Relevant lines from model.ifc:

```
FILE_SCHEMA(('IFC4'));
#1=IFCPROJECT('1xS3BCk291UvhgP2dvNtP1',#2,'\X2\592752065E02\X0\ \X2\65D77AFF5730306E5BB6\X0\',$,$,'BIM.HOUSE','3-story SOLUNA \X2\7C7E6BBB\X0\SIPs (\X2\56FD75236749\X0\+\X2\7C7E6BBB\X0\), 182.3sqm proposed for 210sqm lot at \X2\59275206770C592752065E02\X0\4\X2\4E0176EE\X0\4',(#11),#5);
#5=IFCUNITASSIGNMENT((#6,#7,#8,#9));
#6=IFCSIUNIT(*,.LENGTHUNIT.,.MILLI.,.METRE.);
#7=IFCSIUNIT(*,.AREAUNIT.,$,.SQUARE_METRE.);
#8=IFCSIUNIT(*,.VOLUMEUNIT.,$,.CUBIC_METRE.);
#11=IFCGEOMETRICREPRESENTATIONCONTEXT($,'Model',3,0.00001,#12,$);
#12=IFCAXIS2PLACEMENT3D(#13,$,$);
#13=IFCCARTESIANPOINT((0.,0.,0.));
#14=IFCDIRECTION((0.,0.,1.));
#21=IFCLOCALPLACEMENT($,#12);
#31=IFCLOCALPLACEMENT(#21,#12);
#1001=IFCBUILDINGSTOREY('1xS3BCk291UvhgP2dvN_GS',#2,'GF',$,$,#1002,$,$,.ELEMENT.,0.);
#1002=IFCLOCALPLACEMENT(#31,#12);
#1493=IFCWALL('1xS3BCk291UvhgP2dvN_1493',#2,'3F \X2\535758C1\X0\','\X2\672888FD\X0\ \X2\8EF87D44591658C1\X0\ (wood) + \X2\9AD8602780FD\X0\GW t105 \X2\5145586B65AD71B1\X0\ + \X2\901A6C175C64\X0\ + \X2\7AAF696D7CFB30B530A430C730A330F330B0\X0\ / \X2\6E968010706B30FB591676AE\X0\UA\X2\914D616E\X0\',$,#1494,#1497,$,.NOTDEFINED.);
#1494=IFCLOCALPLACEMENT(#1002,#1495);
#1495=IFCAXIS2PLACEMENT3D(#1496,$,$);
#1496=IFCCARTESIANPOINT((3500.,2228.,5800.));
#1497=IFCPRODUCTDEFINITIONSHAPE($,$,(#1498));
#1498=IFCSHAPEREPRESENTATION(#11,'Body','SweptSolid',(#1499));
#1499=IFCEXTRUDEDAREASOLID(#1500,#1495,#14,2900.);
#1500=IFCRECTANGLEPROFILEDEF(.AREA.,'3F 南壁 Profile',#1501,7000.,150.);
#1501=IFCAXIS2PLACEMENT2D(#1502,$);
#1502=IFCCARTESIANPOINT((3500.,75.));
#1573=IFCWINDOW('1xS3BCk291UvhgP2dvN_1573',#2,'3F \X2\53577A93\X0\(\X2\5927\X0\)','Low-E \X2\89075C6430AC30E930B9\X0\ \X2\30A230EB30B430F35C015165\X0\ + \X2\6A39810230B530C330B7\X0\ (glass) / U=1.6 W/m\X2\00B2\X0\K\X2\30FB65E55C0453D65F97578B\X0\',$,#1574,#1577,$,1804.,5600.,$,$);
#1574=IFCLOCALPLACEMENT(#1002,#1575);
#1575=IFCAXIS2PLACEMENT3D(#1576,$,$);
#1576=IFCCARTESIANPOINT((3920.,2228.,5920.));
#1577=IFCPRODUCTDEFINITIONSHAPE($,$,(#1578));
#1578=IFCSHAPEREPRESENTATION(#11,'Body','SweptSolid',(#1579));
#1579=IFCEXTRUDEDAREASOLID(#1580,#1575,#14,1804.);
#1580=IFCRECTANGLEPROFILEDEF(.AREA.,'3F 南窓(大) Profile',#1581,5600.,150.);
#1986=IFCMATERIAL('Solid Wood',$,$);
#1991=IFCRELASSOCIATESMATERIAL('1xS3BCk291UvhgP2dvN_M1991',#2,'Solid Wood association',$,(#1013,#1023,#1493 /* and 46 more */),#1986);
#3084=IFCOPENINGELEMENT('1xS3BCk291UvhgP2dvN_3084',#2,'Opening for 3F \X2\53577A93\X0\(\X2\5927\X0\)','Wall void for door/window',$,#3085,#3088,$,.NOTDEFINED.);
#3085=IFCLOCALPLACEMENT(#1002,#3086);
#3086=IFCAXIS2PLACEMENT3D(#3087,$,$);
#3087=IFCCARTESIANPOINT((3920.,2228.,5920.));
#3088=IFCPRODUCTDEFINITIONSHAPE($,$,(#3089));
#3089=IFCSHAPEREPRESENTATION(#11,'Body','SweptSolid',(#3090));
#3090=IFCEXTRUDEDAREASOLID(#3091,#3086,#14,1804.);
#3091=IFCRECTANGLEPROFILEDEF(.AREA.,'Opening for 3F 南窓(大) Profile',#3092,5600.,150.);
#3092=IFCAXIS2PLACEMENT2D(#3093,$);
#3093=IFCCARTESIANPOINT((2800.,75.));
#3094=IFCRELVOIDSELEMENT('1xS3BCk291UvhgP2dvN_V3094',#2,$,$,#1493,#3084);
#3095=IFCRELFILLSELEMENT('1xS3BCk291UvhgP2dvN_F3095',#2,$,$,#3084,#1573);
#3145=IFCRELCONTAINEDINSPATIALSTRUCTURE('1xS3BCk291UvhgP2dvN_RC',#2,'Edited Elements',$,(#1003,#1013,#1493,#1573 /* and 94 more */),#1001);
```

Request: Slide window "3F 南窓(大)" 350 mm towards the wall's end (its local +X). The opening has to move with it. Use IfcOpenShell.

```python
import ifcopenshell
import ifcopenshell.api.geometry
import ifcopenshell.util.placement
import ifcopenshell.util.unit

model = ifcopenshell.open("model.ifc")
unit_scale = ifcopenshell.util.unit.calculate_unit_scale(model)

window = model.by_guid("1xS3BCk291UvhgP2dvN_1573")
opening = window.FillsVoids[0].RelatingOpeningElement
wall = opening.VoidsElements[0].RelatingBuildingElement

wall_matrix = ifcopenshell.util.placement.get_local_placement(wall.ObjectPlacement)
shift = wall_matrix[:3, 0] * 0.35 / unit_scale
before = ifcopenshell.util.placement.get_local_placement(window.ObjectPlacement)[:3, 3].copy()

# The window is not placed relative to its opening, so move both.
for product in (opening, window):
    matrix = ifcopenshell.util.placement.get_local_placement(product.ObjectPlacement)
    matrix[:3, 3] += shift
    ifcopenshell.api.geometry.edit_object_placement(model, product=product, matrix=matrix, is_si=False)

after = ifcopenshell.util.placement.get_local_placement(window.ObjectPlacement)[:3, 3]
print("window moved by", (after - before).round(3) + 0.0)

model.write("model_edited.ifc")
```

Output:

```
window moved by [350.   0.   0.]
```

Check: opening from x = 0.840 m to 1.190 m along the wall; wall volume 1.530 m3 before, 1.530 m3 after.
